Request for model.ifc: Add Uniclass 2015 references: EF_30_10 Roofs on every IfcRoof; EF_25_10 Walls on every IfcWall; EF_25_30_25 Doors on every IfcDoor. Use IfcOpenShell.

First a look at what the model holds.

```python
import ifcopenshell

model = ifcopenshell.open("model.ifc")
print(model.schema)
print("classifications:", [c.Name for c in model.by_type("IfcClassification")])
for ifc_class in ("IfcDoor", "IfcRoof", "IfcStair", "IfcWall", "IfcWindow"):
    print(ifc_class, len(model.by_type(ifc_class)))
```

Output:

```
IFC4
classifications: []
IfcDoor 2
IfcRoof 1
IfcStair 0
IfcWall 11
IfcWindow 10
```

```python
import ifcopenshell
import ifcopenshell.api.classification

model = ifcopenshell.open("model.ifc")

system = ifcopenshell.api.classification.add_classification(model, classification="Uniclass 2015")

codes = {
    "IfcRoof": ("EF_30_10", "Roofs"),
    "IfcWall": ("EF_25_10", "Walls"),
    "IfcDoor": ("EF_25_30_25", "Doors"),
}
for ifc_class, (code, name) in codes.items():
    products = model.by_type(ifc_class)
    ifcopenshell.api.classification.add_reference(
        model, products=products, classification=system, identification=code, name=name
    )
    print(code, len(products))

model.write("model-out.ifc")
```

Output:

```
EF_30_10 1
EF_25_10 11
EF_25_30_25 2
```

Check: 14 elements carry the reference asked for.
